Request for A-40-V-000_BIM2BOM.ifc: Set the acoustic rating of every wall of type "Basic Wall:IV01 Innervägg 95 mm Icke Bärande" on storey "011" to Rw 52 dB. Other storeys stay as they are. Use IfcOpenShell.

First a look at what the model holds.

```python
import ifcopenshell
import ifcopenshell.util.element

model = ifcopenshell.open("A-40-V-000_BIM2BOM.ifc")
print(model.schema)
storey = next(s for s in model.by_type("IfcBuildingStorey") if s.Name == "011")
walls = [e for e in ifcopenshell.util.element.get_decomposition(storey) if e.is_a("IfcWall")]
seen = {}
for e in walls:
    element_type = ifcopenshell.util.element.get_type(e)
    key = (element_type.Name if element_type != e and element_type else None, ifcopenshell.util.element.get_pset(e, "Pset_WallCommon", "AcousticRating"))
    seen[key] = seen.get(key, 0) + 1
for (name, value), count in sorted(seen.items(), key=str):
    print(count, "x", name, "|", value)
```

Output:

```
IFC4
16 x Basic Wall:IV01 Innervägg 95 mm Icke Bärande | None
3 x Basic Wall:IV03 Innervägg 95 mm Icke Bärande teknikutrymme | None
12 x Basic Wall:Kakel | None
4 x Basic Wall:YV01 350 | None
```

```python
import ifcopenshell
import ifcopenshell.api.pset
import ifcopenshell.util.element

model = ifcopenshell.open("A-40-V-000_BIM2BOM.ifc")

storey = next(s for s in model.by_type("IfcBuildingStorey") if s.Name == "011")
walls = [e for e in ifcopenshell.util.element.get_decomposition(storey) if e.is_a("IfcWall")]

count = 0
for e in walls:
    element_type = ifcopenshell.util.element.get_type(e)
    if element_type in (None, e) or element_type.Name != "Basic Wall:IV01 Innervägg 95 mm Icke Bärande":
        continue
    # add_pset returns the element's existing set when there is one.
    pset = ifcopenshell.api.pset.add_pset(model, product=e, name="Pset_WallCommon")
    ifcopenshell.api.pset.edit_pset(model, pset=pset, properties={"AcousticRating": "Rw 52 dB"})
    count += 1

print(count, "walls updated")

model.write("A-40-V-000_BIM2BOM-out.ifc")
```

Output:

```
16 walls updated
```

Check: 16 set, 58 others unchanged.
